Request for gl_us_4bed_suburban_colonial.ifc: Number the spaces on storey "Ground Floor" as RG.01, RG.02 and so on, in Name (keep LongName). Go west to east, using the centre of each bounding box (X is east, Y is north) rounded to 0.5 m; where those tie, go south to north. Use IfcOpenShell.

First a look at what the model holds.

```python
import ifcopenshell
import ifcopenshell.util.element
import ifcopenshell.util.placement

model = ifcopenshell.open("gl_us_4bed_suburban_colonial.ifc")
print(model.schema)
storey = next(s for s in model.by_type("IfcBuildingStorey") if s.Name == "Ground Floor")
spaces = [e for e in ifcopenshell.util.element.get_decomposition(storey) if e.is_a("IfcSpace")]
for e in sorted(spaces, key=lambda e: e.id()):
    origin = ifcopenshell.util.placement.get_local_placement(e.ObjectPlacement)[:3, 3]
    print(e.id(), e.Name, e.LongName, origin.round(2) + 0.0, sep=" | ")
```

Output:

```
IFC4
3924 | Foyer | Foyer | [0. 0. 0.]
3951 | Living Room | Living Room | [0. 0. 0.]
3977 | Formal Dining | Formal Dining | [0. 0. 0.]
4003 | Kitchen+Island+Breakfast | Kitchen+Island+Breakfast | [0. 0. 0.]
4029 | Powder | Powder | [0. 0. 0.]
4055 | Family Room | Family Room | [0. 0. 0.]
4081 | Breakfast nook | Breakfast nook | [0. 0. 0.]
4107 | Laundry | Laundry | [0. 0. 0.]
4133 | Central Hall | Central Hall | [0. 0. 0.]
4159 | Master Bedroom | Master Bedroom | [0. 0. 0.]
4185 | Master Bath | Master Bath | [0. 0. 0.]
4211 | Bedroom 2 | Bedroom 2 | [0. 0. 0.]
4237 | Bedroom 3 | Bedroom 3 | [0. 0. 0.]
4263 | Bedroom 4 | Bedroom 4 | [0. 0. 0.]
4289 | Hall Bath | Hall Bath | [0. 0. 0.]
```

```python
import ifcopenshell
import ifcopenshell.geom
import ifcopenshell.util.element
import ifcopenshell.util.shape

model = ifcopenshell.open("gl_us_4bed_suburban_colonial.ifc")
settings = ifcopenshell.geom.settings()
settings.set("use-world-coords", True)


def centre(element):
    shape = ifcopenshell.geom.create_shape(settings, element)
    return ifcopenshell.util.shape.get_bbox_centroid(shape.geometry)


storey = next(s for s in model.by_type("IfcBuildingStorey") if s.Name == "Ground Floor")
spaces = [e for e in ifcopenshell.util.element.get_decomposition(storey) if e.is_a("IfcSpace")]

# Insertion points can sit at a corner or the storey origin, so sort by the geometry (in metres).
centres = {e: centre(e) for e in spaces}
spaces.sort(key=lambda e: (round(centres[e][0] / 0.5), centres[e][1]))

for i, e in enumerate(spaces, start=1):
    number = f"RG.{i:02d}"
    e.Name = number
    print(e.id(), number)

model.write("gl_us_4bed_suburban_colonial_v2.ifc")
```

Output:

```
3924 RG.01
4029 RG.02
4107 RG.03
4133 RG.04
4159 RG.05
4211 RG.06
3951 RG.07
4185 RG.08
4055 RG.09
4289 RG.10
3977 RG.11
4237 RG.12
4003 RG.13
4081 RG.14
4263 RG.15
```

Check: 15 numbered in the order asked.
